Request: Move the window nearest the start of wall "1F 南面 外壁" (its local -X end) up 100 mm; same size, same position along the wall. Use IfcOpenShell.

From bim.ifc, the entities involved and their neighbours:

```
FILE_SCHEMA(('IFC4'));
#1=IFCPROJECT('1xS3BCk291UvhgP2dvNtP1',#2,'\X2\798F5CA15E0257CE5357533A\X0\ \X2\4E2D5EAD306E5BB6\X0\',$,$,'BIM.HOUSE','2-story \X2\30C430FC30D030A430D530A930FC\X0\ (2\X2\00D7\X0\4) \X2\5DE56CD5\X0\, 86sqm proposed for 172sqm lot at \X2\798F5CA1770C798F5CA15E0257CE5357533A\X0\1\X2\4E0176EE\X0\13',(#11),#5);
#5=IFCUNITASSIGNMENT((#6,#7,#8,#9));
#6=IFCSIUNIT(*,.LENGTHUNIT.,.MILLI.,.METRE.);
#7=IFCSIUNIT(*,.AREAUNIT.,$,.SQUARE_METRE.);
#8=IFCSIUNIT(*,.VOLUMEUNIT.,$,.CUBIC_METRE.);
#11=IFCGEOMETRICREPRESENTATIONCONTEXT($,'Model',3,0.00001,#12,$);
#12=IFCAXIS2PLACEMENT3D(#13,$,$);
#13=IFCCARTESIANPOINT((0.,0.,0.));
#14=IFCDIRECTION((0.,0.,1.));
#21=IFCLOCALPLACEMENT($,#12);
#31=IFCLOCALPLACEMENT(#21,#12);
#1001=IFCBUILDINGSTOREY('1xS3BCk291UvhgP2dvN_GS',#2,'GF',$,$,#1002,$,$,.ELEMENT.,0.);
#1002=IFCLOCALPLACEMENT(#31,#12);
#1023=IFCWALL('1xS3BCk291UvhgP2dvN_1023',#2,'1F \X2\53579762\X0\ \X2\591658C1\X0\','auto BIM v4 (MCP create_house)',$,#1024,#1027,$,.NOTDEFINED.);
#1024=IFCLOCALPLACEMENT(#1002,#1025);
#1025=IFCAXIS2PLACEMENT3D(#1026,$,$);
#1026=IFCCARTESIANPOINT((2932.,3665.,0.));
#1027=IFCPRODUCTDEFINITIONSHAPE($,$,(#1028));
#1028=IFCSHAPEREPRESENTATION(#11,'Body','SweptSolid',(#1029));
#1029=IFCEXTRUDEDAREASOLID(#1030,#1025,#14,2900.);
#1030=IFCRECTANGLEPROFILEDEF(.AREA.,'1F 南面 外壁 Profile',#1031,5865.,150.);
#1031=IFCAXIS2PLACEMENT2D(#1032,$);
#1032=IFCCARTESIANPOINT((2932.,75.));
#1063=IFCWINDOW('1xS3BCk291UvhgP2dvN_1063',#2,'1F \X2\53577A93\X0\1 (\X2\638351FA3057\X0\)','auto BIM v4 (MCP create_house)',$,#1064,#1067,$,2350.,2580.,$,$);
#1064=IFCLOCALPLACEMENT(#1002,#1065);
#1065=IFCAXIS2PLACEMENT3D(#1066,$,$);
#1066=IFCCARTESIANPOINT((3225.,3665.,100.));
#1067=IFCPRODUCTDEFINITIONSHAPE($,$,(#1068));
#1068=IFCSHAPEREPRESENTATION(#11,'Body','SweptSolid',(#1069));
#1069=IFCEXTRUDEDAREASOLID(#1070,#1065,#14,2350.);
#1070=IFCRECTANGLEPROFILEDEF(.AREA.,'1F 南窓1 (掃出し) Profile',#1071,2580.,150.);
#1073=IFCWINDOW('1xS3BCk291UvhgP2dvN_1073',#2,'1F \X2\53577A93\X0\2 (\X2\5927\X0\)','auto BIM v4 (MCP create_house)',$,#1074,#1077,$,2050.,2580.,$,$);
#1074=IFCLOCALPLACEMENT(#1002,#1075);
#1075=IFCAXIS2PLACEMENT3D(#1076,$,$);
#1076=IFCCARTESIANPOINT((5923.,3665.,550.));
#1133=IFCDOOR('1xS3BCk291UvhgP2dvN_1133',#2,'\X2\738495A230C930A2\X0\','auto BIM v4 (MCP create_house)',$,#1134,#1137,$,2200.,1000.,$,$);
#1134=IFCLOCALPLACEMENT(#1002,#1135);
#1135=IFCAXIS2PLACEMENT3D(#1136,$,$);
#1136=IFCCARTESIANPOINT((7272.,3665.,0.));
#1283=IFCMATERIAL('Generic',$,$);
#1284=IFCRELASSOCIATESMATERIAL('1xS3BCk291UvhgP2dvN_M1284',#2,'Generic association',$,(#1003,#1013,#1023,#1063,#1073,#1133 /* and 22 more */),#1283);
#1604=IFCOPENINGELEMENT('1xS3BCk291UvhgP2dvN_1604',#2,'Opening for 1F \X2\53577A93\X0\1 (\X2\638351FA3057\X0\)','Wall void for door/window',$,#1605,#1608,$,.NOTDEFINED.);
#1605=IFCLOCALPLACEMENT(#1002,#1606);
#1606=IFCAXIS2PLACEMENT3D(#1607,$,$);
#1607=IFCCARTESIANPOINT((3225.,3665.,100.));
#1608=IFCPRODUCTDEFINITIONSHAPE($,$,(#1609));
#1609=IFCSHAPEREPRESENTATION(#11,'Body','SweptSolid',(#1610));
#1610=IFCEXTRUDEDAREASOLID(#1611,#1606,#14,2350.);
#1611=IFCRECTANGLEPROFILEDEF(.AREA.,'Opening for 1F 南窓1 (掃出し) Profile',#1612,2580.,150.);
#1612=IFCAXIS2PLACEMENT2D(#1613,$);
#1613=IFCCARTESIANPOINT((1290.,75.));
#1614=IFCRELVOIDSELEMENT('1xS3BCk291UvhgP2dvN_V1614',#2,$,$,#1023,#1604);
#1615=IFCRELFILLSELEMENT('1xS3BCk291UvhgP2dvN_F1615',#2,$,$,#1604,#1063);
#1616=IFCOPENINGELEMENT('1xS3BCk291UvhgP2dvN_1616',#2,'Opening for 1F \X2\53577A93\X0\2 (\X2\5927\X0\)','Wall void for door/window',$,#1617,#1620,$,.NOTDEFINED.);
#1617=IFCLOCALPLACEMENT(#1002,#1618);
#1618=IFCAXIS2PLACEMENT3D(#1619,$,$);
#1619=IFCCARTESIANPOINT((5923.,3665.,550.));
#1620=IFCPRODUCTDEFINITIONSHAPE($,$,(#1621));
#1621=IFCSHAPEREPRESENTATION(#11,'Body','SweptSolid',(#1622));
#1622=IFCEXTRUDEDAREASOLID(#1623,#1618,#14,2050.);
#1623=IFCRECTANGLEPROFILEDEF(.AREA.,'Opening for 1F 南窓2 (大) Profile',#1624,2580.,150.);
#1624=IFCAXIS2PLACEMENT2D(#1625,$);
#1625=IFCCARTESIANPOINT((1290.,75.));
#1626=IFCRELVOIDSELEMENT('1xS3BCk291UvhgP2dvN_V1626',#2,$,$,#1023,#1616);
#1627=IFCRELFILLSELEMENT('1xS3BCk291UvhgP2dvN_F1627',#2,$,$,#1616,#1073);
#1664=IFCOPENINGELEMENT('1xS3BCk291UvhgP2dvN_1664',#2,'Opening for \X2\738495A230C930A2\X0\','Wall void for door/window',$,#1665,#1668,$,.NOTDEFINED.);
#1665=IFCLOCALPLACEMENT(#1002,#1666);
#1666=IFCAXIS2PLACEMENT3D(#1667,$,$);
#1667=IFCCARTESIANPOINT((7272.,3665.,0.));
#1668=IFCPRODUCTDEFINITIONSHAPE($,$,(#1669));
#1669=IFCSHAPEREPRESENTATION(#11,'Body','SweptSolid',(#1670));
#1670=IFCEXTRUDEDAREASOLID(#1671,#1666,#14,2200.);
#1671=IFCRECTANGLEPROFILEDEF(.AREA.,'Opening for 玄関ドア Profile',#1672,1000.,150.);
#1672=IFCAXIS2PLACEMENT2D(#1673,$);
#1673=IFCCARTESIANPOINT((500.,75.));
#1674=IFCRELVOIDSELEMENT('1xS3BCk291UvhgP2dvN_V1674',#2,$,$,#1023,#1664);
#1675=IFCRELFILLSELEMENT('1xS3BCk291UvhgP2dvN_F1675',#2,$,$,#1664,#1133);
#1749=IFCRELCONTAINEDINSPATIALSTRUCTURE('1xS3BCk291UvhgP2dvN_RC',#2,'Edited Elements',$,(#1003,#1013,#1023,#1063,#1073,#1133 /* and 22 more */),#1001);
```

```python
import numpy as np
import ifcopenshell
import ifcopenshell.api.geometry
import ifcopenshell.util.placement
import ifcopenshell.util.unit

model = ifcopenshell.open("bim.ifc")
unit_scale = ifcopenshell.util.unit.calculate_unit_scale(model)

window = model.by_guid("1xS3BCk291UvhgP2dvN_1063")
opening = window.FillsVoids[0].RelatingOpeningElement
dz = 0.1 / unit_scale

shift = np.array([0.0, 0.0, dz])
# The window is not placed relative to its opening, so move both.
for product in (opening, window):
    matrix = ifcopenshell.util.placement.get_local_placement(product.ObjectPlacement)
    matrix[:3, 3] += shift
    ifcopenshell.api.geometry.edit_object_placement(model, product=product, matrix=matrix, is_si=False)

print(f"moved by {dz * unit_scale:+.3f} m")

model.write("bim-out.ifc")
```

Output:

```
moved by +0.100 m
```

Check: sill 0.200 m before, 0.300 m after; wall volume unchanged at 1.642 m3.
